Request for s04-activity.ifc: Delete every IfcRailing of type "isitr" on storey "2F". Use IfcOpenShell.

First a look at what the model holds.

```python
import ifcopenshell
import ifcopenshell.util.element

model = ifcopenshell.open("s04-activity.ifc")
print(model.schema)
storey = next(s for s in model.by_type("IfcBuildingStorey") if s.Name == "2F")
railings = [e for e in ifcopenshell.util.element.get_decomposition(storey) if e.is_a("IfcRailing")]
seen = {}
for e in railings:
    element_type = ifcopenshell.util.element.get_type(e)
    name = element_type.Name if element_type not in (None, e) else None
    seen[name] = seen.get(name, 0) + 1
for name, count in sorted(seen.items(), key=str):
    print(count, "x", name)
```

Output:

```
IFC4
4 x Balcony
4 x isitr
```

```python
import ifcopenshell
import ifcopenshell.api.root
import ifcopenshell.util.element

model = ifcopenshell.open("s04-activity.ifc")

storey = next(s for s in model.by_type("IfcBuildingStorey") if s.Name == "2F")
railings = [e for e in ifcopenshell.util.element.get_decomposition(storey) if e.is_a("IfcRailing")]
targets = [e for e in railings if (t := ifcopenshell.util.element.get_type(e)) not in (None, e) and t.Name == "isitr"]

for e in targets:
    ifcopenshell.api.root.remove_product(model, product=e)
print(len(targets), "removed")

model.write("s04-activity-out.ifc")
```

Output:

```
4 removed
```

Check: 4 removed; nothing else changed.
